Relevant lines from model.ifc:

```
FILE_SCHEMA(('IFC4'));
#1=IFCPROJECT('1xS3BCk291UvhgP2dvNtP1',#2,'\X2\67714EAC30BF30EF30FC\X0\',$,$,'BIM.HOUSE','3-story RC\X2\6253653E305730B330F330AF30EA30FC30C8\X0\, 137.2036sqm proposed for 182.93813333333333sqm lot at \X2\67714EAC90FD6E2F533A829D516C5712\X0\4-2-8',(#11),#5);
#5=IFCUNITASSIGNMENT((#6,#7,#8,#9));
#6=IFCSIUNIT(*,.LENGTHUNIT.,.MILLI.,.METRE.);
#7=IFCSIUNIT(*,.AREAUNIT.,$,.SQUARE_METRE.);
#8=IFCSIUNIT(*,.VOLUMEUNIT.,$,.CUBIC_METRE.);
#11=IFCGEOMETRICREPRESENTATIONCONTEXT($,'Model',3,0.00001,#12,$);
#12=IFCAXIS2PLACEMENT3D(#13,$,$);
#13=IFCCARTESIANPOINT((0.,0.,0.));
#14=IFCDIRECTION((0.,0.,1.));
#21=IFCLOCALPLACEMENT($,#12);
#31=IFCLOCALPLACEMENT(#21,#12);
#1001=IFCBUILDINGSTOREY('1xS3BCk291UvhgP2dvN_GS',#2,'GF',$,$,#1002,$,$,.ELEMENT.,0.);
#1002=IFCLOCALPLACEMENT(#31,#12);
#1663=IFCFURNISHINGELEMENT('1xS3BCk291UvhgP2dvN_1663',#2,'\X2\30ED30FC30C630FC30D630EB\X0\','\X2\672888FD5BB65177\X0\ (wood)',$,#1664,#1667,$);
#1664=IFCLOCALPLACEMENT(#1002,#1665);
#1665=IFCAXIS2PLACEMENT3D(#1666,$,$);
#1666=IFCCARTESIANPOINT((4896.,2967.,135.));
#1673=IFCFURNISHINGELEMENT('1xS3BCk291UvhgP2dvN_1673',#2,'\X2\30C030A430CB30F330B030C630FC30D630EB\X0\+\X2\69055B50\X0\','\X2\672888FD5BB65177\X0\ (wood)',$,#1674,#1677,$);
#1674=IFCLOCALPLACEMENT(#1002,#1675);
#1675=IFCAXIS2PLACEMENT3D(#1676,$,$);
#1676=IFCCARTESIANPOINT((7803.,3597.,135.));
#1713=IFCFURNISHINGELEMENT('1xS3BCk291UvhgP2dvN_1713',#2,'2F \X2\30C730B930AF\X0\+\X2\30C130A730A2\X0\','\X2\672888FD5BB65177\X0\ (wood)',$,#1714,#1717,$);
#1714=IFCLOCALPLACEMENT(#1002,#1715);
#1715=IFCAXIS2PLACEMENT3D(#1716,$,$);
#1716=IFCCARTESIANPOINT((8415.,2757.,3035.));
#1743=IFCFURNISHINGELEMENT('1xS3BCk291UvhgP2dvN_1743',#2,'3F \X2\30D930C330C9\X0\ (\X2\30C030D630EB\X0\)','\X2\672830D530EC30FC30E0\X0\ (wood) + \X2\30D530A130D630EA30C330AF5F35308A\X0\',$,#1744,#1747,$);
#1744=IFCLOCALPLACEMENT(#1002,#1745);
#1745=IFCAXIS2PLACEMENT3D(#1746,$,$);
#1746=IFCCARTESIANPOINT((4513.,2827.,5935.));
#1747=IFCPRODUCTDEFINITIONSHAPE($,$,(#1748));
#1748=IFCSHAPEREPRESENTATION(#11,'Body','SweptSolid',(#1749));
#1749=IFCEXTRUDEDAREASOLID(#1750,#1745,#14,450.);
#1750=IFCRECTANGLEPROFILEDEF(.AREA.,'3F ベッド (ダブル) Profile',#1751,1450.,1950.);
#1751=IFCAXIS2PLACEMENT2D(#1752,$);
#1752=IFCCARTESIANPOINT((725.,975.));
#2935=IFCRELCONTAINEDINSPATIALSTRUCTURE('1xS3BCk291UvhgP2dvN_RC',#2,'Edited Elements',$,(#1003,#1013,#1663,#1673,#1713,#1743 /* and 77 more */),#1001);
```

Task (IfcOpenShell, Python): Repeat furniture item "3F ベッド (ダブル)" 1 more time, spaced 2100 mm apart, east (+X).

```python
import numpy as np
import ifcopenshell
import ifcopenshell.api.geometry
import ifcopenshell.api.root
import ifcopenshell.util.element
import ifcopenshell.util.placement
import ifcopenshell.util.unit

model = ifcopenshell.open("model.ifc")
unit_scale = ifcopenshell.util.unit.calculate_unit_scale(model)


def reuse_history(source, copy):
    """copy_class also copies each property set's owner history, people and application; keep the originals."""
    for rel in copy.IsDefinedBy:
        if rel.is_a("IfcRelDefinesByProperties") and (history := rel.RelatingPropertyDefinition.OwnerHistory):
            rel.RelatingPropertyDefinition.OwnerHistory = source.OwnerHistory
            ifcopenshell.util.element.remove_deep2(model, history)


source = model.by_guid("1xS3BCk291UvhgP2dvN_1743")
base = ifcopenshell.util.placement.get_local_placement(source.ObjectPlacement)
step = np.array([1.0, 0.0, 0.0]) * 2.1 / unit_scale

for i in range(1, 2):
    copy = ifcopenshell.api.root.copy_class(model, product=source)
    copy.Representation = ifcopenshell.util.element.copy_deep(
        model, source.Representation, exclude=["IfcGeometricRepresentationContext", "IfcRepresentationMap"]
    )
    reuse_history(source, copy)
    matrix = base.copy()
    matrix[:3, 3] += i * step
    print("added at", matrix[:3, 3].round(3) + 0.0)
    ifcopenshell.api.geometry.edit_object_placement(model, product=copy, matrix=matrix, is_si=False)

model.write("model-out.ifc")
```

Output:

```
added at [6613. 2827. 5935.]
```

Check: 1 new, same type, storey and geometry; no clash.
